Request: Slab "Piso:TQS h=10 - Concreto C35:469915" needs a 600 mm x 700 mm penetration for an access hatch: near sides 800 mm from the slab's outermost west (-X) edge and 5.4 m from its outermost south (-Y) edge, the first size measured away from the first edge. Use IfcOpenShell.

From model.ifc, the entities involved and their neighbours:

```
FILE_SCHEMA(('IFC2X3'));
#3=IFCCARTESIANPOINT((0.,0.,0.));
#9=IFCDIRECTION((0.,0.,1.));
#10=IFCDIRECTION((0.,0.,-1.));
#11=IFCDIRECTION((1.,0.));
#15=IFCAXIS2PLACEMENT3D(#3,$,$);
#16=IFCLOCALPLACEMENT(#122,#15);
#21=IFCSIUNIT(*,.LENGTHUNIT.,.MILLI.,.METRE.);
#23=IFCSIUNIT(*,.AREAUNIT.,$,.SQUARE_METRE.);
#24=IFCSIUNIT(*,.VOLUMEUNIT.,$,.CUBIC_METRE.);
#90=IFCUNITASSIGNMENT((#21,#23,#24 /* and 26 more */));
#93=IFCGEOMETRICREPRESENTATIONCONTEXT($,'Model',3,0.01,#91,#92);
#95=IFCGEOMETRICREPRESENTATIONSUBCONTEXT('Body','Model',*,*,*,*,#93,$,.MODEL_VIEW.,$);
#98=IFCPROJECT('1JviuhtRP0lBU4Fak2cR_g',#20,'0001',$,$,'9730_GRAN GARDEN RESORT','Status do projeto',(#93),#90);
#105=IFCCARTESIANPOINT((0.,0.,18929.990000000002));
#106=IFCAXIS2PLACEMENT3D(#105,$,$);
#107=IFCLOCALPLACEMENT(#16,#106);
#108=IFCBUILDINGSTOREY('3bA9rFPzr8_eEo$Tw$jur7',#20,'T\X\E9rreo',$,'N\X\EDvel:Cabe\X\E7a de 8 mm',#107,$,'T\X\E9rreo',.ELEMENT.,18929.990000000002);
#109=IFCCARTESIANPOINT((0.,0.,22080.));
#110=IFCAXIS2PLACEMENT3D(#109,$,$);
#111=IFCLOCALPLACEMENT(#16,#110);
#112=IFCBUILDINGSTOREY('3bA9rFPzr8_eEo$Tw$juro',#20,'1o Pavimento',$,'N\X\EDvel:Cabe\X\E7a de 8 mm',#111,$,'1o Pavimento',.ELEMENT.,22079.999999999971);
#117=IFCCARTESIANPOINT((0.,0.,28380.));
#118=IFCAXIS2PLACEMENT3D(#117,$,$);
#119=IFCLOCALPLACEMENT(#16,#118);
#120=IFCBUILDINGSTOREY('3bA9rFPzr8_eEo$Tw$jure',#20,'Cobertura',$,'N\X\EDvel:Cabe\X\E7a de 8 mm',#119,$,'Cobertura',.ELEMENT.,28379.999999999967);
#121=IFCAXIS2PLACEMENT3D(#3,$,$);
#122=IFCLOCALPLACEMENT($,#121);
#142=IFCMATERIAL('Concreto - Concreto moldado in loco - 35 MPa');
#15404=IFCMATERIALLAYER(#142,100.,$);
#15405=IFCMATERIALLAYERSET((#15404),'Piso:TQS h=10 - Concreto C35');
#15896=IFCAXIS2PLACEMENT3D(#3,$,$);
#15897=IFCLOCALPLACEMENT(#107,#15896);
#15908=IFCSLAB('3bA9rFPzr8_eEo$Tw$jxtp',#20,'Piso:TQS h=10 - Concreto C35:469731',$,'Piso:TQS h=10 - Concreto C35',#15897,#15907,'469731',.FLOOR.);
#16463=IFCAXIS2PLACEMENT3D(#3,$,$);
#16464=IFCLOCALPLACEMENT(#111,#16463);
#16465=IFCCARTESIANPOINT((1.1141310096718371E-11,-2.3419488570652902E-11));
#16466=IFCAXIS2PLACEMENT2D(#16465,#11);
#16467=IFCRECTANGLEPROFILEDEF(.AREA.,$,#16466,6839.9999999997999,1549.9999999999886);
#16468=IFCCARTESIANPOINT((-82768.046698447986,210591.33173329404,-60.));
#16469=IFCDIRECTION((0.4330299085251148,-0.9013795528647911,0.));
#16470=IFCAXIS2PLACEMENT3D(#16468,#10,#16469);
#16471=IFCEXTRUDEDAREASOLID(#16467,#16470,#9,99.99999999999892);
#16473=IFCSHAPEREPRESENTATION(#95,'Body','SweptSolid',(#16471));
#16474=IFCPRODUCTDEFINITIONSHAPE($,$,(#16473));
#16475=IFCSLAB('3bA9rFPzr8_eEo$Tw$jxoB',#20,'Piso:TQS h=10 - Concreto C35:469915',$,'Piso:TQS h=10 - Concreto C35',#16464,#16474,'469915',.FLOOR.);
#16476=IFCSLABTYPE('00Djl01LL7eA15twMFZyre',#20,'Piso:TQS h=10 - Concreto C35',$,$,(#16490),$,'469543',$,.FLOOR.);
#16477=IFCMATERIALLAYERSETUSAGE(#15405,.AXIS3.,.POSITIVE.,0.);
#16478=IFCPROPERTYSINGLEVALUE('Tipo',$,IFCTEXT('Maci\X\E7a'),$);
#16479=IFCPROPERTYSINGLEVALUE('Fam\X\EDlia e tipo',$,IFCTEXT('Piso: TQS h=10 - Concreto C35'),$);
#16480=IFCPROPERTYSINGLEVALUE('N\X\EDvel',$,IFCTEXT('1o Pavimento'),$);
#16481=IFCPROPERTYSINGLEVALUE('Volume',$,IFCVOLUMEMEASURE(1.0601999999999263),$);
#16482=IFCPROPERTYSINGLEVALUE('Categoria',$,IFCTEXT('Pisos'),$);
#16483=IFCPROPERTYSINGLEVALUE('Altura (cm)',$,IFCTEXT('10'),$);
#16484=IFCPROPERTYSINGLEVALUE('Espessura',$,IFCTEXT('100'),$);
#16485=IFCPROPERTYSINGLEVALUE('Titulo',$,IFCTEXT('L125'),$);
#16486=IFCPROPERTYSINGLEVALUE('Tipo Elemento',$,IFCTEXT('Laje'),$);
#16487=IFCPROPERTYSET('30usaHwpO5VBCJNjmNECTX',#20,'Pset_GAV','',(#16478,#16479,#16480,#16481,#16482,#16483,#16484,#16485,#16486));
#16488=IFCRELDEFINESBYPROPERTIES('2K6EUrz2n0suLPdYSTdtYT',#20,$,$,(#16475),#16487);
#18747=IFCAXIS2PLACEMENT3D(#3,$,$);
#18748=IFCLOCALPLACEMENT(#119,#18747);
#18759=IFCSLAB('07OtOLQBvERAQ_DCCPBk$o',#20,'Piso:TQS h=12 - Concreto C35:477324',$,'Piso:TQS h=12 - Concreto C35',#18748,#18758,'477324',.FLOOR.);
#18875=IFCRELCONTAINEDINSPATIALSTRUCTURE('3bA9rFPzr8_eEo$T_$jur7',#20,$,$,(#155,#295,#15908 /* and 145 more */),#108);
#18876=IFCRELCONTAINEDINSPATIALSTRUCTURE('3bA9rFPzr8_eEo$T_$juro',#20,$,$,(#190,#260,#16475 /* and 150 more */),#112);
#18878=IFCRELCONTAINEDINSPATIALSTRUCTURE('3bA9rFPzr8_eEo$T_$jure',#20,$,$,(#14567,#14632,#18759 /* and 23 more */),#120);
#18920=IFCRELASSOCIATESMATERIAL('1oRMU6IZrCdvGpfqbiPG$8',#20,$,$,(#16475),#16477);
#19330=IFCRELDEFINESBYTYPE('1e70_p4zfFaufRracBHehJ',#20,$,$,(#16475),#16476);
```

```python
import numpy as np
import ifcopenshell
import ifcopenshell.api.feature
import ifcopenshell.api.geometry
import ifcopenshell.api.pset
import ifcopenshell.api.root
import ifcopenshell.geom
import ifcopenshell.util.element
import ifcopenshell.util.placement
import ifcopenshell.util.representation
import ifcopenshell.util.shape
import ifcopenshell.util.unit

model = ifcopenshell.open("model.ifc")
unit_scale = ifcopenshell.util.unit.calculate_unit_scale(model)
volume_scale = ifcopenshell.util.unit.calculate_unit_scale(model, "VOLUMEUNIT")
settings = ifcopenshell.geom.settings()


def volume(element):
    """Net volume in cubic metres, openings subtracted."""
    shape = ifcopenshell.geom.create_shape(settings, element)
    return ifcopenshell.util.shape.get_volume(shape.geometry)


slab = model.by_guid("3bA9rFPzr8_eEo$Tw$jxoB")
before = volume(slab)

# Extent in the slab's own axes, in metres. The edges named are its -X and -Y sides.
slab_shape = ifcopenshell.geom.create_shape(settings, slab)
vertices = ifcopenshell.util.shape.get_vertices(slab_shape.geometry)
x_min, y_min, bottom = vertices.min(axis=0)
top = vertices[:, 2].max()

opening = ifcopenshell.api.root.create_entity(model, ifc_class="IfcOpeningElement", name="Access hatch opening")
context = ifcopenshell.util.representation.get_context(model, "Model", "Body", "MODEL_VIEW")
width, depth = 0.6, 0.7
outline = [(0.0, 0.0), (width, 0.0), (width, depth), (0.0, depth), (0.0, 0.0)]
# Overshoot both faces by 50 mm so the cut is clean.
shape = ifcopenshell.api.geometry.add_slab_representation(
    model, context=context, depth=top - bottom + 0.1, polyline=outline
)
ifcopenshell.api.geometry.assign_representation(model, product=opening, representation=shape)

matrix = ifcopenshell.util.placement.get_local_placement(slab.ObjectPlacement)
matrix[:, 3] = matrix @ np.append(np.array([x_min + 0.8, y_min + 5.4, bottom - 0.05]) / unit_scale, 1.0)
ifcopenshell.api.geometry.edit_object_placement(model, product=opening, matrix=matrix, is_si=False)
ifcopenshell.api.feature.add_feature(model, feature=opening, element=slab)

after = volume(slab)

# Update the slab's stored quantities.
pset = model.by_id(ifcopenshell.util.element.get_pset(slab, "Pset_GAV", should_inherit=False)["id"])
ifcopenshell.api.pset.edit_pset(model, pset=pset, properties={
    "Volume": model.create_entity("IfcVolumeMeasure", after / volume_scale),
})

print(f"slab volume {before:.3f} -> {after:.3f} m3")

model.write("model_rev.ifc")
```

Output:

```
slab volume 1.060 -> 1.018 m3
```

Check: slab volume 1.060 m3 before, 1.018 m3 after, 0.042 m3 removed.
